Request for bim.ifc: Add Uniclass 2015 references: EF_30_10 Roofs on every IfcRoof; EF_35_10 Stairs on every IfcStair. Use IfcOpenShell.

First a look at what the model holds.

```python
import ifcopenshell

model = ifcopenshell.open("bim.ifc")
print(model.schema)
print("classifications:", [c.Name for c in model.by_type("IfcClassification")])
for ifc_class in ("IfcDoor", "IfcRoof", "IfcStair", "IfcWall", "IfcWindow"):
    print(ifc_class, len(model.by_type(ifc_class)))
```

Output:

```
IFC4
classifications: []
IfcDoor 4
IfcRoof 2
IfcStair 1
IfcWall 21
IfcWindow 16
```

```python
import ifcopenshell
import ifcopenshell.api.classification

model = ifcopenshell.open("bim.ifc")

system = ifcopenshell.api.classification.add_classification(model, classification="Uniclass 2015")

codes = {
    "IfcRoof": ("EF_30_10", "Roofs"),
    "IfcStair": ("EF_35_10", "Stairs"),
}
for ifc_class, (code, name) in codes.items():
    products = model.by_type(ifc_class)
    ifcopenshell.api.classification.add_reference(
        model, products=products, classification=system, identification=code, name=name
    )
    print(code, len(products))

model.write("bim_edited.ifc")
```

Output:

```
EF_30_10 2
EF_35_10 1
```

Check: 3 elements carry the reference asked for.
